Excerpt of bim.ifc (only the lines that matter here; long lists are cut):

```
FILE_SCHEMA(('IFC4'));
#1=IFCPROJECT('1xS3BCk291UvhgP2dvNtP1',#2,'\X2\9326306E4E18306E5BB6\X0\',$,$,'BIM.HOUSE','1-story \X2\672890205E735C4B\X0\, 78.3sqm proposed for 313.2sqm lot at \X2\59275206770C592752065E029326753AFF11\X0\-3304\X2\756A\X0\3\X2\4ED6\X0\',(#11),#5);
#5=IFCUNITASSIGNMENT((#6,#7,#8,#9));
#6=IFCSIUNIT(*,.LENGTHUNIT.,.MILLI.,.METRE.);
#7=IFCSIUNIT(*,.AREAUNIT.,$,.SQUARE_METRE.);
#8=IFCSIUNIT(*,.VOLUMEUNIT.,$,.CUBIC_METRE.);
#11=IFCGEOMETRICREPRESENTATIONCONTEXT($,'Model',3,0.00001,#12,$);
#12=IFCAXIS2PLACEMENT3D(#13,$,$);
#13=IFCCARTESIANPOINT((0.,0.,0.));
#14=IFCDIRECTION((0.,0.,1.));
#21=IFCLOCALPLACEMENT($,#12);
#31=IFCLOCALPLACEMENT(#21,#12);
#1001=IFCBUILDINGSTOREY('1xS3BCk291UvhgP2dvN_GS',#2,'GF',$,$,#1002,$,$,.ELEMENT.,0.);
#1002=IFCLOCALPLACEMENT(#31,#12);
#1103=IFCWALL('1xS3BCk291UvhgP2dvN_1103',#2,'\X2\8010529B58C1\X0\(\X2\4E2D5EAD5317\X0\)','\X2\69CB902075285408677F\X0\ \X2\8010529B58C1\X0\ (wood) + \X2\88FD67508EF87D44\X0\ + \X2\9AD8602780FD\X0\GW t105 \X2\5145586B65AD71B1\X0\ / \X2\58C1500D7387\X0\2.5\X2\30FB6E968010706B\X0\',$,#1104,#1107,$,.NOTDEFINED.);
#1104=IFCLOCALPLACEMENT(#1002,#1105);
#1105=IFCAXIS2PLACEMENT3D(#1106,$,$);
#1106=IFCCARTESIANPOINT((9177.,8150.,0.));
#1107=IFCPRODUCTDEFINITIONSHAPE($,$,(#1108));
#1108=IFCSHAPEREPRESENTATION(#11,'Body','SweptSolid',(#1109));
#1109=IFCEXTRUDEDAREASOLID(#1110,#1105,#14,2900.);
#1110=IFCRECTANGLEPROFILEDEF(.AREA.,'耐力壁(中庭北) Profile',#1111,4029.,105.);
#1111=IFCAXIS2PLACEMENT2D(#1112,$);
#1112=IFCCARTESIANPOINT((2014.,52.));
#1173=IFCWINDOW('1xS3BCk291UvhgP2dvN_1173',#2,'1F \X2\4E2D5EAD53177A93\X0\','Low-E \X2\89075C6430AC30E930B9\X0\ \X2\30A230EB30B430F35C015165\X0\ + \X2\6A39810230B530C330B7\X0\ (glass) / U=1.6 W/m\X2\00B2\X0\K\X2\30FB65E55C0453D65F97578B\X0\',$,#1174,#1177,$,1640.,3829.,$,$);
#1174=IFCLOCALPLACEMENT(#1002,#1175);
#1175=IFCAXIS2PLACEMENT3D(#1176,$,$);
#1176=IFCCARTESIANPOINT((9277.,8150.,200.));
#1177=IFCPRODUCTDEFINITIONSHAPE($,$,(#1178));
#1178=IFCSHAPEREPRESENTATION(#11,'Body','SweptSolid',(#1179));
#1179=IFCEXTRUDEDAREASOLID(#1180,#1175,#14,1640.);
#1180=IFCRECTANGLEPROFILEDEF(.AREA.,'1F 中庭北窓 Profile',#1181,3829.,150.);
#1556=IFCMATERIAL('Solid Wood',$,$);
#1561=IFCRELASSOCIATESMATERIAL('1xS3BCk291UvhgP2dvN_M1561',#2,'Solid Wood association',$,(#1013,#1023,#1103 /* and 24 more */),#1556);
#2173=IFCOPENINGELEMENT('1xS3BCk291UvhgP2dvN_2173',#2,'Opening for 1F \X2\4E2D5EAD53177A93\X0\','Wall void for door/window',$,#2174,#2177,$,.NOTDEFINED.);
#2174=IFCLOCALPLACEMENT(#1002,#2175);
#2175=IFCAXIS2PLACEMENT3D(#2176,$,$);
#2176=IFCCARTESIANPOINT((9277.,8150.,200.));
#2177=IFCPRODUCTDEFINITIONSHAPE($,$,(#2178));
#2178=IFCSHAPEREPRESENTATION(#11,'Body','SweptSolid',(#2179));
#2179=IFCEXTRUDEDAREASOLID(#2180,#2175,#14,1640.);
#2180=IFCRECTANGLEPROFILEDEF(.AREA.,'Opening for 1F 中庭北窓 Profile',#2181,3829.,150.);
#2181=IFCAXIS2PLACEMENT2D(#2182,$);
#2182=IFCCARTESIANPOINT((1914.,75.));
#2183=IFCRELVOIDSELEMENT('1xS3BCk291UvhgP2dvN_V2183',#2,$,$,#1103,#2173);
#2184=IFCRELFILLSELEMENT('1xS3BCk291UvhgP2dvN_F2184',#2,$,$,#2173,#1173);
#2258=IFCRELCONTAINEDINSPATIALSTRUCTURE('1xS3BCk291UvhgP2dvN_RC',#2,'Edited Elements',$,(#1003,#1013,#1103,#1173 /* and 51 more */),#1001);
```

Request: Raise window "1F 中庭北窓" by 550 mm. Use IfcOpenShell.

```python
import numpy as np
import ifcopenshell
import ifcopenshell.api.geometry
import ifcopenshell.util.placement
import ifcopenshell.util.unit

model = ifcopenshell.open("bim.ifc")
unit_scale = ifcopenshell.util.unit.calculate_unit_scale(model)

window = model.by_id(1173)
opening = window.FillsVoids[0].RelatingOpeningElement
dz = 0.55 / unit_scale

shift = np.array([0.0, 0.0, dz])
# The window is not placed relative to its opening, so move both.
for product in (opening, window):
    matrix = ifcopenshell.util.placement.get_local_placement(product.ObjectPlacement)
    matrix[:3, 3] += shift
    ifcopenshell.api.geometry.edit_object_placement(model, product=product, matrix=matrix, is_si=False)

print(f"moved by {dz * unit_scale:+.3f} m")

model.write("bim_v2.ifc")
```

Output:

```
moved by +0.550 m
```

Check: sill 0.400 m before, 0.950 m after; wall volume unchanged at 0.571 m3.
